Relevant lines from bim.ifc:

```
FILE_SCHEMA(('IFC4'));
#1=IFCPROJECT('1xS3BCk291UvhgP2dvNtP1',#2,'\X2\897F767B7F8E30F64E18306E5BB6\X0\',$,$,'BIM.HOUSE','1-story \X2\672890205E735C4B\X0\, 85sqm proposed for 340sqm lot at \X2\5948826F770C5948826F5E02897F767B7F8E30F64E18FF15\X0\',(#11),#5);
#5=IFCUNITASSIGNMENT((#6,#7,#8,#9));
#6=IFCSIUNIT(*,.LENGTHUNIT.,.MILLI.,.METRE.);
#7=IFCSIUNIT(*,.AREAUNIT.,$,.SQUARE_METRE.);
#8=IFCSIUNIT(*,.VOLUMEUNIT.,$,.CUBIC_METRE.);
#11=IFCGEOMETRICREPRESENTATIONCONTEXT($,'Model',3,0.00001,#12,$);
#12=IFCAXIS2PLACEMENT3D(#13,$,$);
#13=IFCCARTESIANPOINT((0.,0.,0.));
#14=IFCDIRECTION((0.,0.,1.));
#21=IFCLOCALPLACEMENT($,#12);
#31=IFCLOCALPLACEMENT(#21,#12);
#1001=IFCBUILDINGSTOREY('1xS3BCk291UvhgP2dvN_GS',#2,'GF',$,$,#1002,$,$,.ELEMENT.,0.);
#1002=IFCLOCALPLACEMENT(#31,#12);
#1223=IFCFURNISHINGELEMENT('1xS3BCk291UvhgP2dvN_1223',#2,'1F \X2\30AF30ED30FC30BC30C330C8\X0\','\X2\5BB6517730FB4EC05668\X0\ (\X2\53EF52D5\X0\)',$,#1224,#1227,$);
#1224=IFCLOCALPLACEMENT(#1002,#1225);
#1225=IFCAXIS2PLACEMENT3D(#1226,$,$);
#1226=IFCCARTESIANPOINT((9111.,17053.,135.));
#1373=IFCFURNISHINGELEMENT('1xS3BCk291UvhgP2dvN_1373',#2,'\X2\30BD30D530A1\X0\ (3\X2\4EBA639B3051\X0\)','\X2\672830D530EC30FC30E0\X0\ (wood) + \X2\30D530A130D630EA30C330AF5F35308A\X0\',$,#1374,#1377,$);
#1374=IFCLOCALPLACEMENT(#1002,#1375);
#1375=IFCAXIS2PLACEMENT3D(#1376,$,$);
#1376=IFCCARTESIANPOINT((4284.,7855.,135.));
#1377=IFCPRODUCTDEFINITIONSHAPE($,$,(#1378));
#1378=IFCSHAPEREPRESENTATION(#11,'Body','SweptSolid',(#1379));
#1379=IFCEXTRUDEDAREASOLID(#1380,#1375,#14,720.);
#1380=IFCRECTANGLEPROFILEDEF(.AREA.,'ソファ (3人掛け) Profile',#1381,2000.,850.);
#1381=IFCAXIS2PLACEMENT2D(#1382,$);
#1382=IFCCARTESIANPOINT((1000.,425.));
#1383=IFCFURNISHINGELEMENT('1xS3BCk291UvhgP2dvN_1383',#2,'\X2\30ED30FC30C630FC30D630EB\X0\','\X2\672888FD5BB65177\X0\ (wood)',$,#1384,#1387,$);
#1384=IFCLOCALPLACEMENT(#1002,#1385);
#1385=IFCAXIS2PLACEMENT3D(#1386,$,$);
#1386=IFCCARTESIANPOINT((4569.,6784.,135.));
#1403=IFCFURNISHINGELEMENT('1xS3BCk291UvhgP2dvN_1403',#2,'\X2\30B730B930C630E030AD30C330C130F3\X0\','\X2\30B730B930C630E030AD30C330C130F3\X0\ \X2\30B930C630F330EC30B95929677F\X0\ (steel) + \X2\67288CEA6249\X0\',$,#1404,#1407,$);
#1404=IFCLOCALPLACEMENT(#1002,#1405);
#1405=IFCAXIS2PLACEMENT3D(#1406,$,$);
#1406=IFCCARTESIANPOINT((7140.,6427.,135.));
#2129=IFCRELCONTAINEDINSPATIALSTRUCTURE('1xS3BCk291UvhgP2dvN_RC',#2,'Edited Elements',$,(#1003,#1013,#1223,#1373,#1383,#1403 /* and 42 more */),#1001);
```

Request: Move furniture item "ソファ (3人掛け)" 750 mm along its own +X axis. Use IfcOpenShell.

```python
import ifcopenshell
import ifcopenshell.api.geometry
import ifcopenshell.util.placement
import ifcopenshell.util.unit

model = ifcopenshell.open("bim.ifc")
unit_scale = ifcopenshell.util.unit.calculate_unit_scale(model)

item = model.by_id(1373)
matrix = ifcopenshell.util.placement.get_local_placement(item.ObjectPlacement)
matrix[:3, 3] += matrix[:3, 0] * 0.75 / unit_scale
ifcopenshell.api.geometry.edit_object_placement(model, product=item, matrix=matrix, is_si=False)

print(ifcopenshell.util.placement.get_local_placement(item.ObjectPlacement).round(3) + 0.0)

model.write("bim-out.ifc")
```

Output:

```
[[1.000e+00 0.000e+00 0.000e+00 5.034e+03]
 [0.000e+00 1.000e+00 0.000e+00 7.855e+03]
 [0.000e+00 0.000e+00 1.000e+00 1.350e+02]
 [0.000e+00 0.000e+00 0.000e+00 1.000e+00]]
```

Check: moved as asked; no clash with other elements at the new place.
